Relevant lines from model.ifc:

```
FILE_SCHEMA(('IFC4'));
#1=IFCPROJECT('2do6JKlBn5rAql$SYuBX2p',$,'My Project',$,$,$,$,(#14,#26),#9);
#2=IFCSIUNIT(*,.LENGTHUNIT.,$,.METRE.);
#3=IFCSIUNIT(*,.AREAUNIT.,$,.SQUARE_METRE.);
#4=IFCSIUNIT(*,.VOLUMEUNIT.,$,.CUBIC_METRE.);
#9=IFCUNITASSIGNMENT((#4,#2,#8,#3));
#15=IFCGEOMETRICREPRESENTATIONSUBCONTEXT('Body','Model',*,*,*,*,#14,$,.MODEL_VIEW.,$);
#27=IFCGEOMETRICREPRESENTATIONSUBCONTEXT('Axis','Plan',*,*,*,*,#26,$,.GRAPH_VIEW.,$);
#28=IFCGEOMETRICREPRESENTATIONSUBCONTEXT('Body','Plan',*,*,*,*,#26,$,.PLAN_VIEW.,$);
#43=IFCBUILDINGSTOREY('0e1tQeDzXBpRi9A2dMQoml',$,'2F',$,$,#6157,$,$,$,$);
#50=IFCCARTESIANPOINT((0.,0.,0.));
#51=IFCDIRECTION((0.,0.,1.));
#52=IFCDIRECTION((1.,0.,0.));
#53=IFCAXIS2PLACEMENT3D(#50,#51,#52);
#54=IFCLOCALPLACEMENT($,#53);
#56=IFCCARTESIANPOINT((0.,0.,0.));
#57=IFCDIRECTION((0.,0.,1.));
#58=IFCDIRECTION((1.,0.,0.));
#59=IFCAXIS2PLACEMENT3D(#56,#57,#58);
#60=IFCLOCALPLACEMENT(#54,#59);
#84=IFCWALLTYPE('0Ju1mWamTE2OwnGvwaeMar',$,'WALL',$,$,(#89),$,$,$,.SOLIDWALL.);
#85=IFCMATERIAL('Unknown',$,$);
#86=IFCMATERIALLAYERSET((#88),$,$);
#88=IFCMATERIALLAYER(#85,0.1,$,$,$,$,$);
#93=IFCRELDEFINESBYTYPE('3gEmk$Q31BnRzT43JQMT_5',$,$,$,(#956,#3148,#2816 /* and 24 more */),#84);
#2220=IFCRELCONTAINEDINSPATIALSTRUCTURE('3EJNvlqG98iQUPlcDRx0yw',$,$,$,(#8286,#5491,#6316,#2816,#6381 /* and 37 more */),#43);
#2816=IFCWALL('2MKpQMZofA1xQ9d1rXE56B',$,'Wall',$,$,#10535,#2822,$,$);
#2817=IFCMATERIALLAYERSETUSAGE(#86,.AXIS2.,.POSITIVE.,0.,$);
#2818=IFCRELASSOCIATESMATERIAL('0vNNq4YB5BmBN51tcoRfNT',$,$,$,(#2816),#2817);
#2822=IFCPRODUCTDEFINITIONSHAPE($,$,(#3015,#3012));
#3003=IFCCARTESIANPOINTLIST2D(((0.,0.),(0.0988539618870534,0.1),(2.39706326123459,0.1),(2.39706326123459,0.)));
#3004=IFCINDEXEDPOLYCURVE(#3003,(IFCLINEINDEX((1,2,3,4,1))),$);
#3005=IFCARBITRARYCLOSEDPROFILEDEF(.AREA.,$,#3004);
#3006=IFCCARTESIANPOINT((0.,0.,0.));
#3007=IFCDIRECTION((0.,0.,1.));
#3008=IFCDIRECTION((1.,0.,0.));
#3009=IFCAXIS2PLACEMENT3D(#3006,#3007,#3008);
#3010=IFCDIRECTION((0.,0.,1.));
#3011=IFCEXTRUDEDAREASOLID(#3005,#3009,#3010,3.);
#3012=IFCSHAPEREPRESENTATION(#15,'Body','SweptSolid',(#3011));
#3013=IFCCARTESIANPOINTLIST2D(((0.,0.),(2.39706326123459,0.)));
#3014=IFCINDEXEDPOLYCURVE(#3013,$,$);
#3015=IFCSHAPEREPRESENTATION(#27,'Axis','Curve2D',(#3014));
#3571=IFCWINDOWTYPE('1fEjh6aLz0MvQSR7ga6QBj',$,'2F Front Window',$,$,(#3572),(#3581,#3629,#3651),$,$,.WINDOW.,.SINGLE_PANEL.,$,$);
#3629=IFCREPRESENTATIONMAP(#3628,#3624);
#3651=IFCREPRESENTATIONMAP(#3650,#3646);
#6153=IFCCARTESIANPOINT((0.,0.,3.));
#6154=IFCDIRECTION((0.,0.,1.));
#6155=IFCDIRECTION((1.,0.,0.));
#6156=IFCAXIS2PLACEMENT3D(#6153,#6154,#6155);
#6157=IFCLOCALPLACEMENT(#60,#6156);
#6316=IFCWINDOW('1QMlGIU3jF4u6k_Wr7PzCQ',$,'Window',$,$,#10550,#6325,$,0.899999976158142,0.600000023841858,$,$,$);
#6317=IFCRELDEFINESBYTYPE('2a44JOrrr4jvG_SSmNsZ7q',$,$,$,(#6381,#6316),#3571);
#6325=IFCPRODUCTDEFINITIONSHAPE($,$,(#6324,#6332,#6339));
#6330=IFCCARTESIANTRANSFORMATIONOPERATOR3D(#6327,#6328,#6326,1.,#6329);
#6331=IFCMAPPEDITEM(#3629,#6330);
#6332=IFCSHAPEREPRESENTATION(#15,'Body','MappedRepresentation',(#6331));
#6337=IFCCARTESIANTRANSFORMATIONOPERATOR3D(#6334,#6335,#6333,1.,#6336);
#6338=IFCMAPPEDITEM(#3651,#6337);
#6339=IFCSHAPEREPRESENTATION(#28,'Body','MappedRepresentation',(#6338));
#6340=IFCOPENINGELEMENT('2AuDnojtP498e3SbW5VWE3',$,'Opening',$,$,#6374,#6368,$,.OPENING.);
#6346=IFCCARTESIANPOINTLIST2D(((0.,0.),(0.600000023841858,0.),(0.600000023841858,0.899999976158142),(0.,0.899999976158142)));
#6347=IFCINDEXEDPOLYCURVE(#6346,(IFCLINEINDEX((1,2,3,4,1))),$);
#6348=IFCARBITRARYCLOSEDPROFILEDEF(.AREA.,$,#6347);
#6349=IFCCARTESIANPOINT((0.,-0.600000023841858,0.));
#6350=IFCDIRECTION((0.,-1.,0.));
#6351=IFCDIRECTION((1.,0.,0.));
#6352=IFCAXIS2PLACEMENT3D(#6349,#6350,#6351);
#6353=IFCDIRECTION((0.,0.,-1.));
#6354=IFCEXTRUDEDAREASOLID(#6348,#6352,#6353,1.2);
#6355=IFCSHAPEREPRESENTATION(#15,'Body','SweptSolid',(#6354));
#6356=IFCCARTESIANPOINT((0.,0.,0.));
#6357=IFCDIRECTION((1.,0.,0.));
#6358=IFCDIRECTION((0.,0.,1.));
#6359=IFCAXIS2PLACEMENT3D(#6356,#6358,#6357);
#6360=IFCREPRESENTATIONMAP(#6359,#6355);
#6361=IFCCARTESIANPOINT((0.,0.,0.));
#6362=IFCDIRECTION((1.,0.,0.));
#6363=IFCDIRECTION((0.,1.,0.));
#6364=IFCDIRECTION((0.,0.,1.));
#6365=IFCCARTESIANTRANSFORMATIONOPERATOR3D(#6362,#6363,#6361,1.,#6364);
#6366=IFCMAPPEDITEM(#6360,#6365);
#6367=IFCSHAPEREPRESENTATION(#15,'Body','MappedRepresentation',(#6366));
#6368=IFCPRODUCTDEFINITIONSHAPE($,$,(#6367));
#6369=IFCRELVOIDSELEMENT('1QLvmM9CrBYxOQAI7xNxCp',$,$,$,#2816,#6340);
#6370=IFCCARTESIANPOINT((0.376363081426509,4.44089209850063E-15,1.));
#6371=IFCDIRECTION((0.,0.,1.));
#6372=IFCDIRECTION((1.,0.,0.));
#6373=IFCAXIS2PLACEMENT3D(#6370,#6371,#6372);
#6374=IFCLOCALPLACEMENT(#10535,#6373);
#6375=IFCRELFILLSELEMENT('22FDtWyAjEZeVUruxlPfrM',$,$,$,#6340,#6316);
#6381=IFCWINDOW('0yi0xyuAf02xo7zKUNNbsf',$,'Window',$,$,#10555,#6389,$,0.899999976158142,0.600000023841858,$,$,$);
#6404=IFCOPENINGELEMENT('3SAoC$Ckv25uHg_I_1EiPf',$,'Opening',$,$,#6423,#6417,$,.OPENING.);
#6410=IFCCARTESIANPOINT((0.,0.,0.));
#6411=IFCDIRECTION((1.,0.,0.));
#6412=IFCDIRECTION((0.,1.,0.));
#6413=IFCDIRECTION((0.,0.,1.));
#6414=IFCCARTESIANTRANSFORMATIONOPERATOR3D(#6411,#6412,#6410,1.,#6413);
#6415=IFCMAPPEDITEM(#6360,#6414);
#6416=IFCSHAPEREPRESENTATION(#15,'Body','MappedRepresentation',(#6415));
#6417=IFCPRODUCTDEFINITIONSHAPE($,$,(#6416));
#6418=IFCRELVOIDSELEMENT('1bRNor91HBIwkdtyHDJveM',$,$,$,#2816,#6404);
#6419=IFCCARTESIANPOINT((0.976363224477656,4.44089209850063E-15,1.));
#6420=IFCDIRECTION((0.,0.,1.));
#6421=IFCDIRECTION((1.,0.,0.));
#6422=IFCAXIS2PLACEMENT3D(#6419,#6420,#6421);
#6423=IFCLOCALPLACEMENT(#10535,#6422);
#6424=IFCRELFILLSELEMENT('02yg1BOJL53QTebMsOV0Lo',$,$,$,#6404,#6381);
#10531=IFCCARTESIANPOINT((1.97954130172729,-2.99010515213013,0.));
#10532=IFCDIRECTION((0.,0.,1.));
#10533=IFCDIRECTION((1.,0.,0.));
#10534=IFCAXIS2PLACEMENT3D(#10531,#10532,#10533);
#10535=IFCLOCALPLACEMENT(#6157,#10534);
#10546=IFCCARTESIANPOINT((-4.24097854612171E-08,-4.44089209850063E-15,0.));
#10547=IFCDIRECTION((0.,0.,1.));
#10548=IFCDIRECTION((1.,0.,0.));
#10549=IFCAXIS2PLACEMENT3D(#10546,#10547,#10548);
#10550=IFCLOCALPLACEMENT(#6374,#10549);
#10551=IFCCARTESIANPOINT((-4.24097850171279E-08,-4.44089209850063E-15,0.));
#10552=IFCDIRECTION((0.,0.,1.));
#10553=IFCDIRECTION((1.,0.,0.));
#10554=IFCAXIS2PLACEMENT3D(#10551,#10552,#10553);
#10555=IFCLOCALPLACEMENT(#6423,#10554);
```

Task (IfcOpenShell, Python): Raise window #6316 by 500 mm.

```python
import numpy as np
import ifcopenshell
import ifcopenshell.api.geometry
import ifcopenshell.util.placement
import ifcopenshell.util.unit

model = ifcopenshell.open("model.ifc")
unit_scale = ifcopenshell.util.unit.calculate_unit_scale(model)

window = model.by_id(6316)
opening = window.FillsVoids[0].RelatingOpeningElement
dz = 0.5 / unit_scale

shift = np.array([0.0, 0.0, dz])
# The window is placed relative to its opening, so it follows when the opening moves.
matrix = ifcopenshell.util.placement.get_local_placement(opening.ObjectPlacement)
matrix[:3, 3] += shift
ifcopenshell.api.geometry.edit_object_placement(
    model, product=opening, matrix=matrix, is_si=False, should_transform_children=True
)

print(f"moved by {dz * unit_scale:+.3f} m")

model.write("model_edited.ifc")
```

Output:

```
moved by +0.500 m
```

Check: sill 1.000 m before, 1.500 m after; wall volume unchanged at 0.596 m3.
